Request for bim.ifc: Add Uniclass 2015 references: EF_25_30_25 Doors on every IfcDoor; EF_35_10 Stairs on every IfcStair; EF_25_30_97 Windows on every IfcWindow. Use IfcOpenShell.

First a look at what the model holds.

```python
import ifcopenshell

model = ifcopenshell.open("bim.ifc")
print(model.schema)
print("classifications:", [c.Name for c in model.by_type("IfcClassification")])
for ifc_class in ("IfcDoor", "IfcRoof", "IfcStair", "IfcWall", "IfcWindow"):
    print(ifc_class, len(model.by_type(ifc_class)))
```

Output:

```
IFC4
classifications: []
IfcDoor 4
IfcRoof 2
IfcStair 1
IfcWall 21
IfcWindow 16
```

```python
import ifcopenshell
import ifcopenshell.api.classification

model = ifcopenshell.open("bim.ifc")

system = ifcopenshell.api.classification.add_classification(model, classification="Uniclass 2015")

codes = {
    "IfcDoor": ("EF_25_30_25", "Doors"),
    "IfcStair": ("EF_35_10", "Stairs"),
    "IfcWindow": ("EF_25_30_97", "Windows"),
}
for ifc_class, (code, name) in codes.items():
    products = model.by_type(ifc_class)
    ifcopenshell.api.classification.add_reference(
        model, products=products, classification=system, identification=code, name=name
    )
    print(code, len(products))

model.write("bim_v2.ifc")
```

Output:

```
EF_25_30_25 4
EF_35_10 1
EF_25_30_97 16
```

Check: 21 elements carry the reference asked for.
